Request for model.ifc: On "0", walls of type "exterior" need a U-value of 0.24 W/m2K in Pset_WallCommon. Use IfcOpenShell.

First a look at what the model holds.

```python
import ifcopenshell
import ifcopenshell.util.element

model = ifcopenshell.open("model.ifc")
print(model.schema)
storey = next(s for s in model.by_type("IfcBuildingStorey") if s.Name == "0")
walls = [e for e in ifcopenshell.util.element.get_decomposition(storey) if e.is_a("IfcWall")]
seen = {}
for e in walls:
    element_type = ifcopenshell.util.element.get_type(e)
    key = (element_type.Name if element_type != e and element_type else None, ifcopenshell.util.element.get_pset(e, "Pset_WallCommon", "ThermalTransmittance"))
    seen[key] = seen.get(key, 0) + 1
for (name, value), count in sorted(seen.items(), key=str):
    print(count, "x", name, "|", value)
```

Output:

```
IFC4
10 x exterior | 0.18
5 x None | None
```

```python
import ifcopenshell
import ifcopenshell.api.pset
import ifcopenshell.util.element

model = ifcopenshell.open("model.ifc")

storey = next(s for s in model.by_type("IfcBuildingStorey") if s.Name == "0")
walls = [e for e in ifcopenshell.util.element.get_decomposition(storey) if e.is_a("IfcWall")]

count = 0
for e in walls:
    element_type = ifcopenshell.util.element.get_type(e)
    if element_type in (None, e) or element_type.Name != "exterior":
        continue
    # add_pset returns the element's existing set when there is one.
    pset = ifcopenshell.api.pset.add_pset(model, product=e, name="Pset_WallCommon")
    ifcopenshell.api.pset.edit_pset(model, pset=pset, properties={"ThermalTransmittance": 0.24})
    count += 1

print(count, "walls updated")

model.write("model_edited.ifc")
```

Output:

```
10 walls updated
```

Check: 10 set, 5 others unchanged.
